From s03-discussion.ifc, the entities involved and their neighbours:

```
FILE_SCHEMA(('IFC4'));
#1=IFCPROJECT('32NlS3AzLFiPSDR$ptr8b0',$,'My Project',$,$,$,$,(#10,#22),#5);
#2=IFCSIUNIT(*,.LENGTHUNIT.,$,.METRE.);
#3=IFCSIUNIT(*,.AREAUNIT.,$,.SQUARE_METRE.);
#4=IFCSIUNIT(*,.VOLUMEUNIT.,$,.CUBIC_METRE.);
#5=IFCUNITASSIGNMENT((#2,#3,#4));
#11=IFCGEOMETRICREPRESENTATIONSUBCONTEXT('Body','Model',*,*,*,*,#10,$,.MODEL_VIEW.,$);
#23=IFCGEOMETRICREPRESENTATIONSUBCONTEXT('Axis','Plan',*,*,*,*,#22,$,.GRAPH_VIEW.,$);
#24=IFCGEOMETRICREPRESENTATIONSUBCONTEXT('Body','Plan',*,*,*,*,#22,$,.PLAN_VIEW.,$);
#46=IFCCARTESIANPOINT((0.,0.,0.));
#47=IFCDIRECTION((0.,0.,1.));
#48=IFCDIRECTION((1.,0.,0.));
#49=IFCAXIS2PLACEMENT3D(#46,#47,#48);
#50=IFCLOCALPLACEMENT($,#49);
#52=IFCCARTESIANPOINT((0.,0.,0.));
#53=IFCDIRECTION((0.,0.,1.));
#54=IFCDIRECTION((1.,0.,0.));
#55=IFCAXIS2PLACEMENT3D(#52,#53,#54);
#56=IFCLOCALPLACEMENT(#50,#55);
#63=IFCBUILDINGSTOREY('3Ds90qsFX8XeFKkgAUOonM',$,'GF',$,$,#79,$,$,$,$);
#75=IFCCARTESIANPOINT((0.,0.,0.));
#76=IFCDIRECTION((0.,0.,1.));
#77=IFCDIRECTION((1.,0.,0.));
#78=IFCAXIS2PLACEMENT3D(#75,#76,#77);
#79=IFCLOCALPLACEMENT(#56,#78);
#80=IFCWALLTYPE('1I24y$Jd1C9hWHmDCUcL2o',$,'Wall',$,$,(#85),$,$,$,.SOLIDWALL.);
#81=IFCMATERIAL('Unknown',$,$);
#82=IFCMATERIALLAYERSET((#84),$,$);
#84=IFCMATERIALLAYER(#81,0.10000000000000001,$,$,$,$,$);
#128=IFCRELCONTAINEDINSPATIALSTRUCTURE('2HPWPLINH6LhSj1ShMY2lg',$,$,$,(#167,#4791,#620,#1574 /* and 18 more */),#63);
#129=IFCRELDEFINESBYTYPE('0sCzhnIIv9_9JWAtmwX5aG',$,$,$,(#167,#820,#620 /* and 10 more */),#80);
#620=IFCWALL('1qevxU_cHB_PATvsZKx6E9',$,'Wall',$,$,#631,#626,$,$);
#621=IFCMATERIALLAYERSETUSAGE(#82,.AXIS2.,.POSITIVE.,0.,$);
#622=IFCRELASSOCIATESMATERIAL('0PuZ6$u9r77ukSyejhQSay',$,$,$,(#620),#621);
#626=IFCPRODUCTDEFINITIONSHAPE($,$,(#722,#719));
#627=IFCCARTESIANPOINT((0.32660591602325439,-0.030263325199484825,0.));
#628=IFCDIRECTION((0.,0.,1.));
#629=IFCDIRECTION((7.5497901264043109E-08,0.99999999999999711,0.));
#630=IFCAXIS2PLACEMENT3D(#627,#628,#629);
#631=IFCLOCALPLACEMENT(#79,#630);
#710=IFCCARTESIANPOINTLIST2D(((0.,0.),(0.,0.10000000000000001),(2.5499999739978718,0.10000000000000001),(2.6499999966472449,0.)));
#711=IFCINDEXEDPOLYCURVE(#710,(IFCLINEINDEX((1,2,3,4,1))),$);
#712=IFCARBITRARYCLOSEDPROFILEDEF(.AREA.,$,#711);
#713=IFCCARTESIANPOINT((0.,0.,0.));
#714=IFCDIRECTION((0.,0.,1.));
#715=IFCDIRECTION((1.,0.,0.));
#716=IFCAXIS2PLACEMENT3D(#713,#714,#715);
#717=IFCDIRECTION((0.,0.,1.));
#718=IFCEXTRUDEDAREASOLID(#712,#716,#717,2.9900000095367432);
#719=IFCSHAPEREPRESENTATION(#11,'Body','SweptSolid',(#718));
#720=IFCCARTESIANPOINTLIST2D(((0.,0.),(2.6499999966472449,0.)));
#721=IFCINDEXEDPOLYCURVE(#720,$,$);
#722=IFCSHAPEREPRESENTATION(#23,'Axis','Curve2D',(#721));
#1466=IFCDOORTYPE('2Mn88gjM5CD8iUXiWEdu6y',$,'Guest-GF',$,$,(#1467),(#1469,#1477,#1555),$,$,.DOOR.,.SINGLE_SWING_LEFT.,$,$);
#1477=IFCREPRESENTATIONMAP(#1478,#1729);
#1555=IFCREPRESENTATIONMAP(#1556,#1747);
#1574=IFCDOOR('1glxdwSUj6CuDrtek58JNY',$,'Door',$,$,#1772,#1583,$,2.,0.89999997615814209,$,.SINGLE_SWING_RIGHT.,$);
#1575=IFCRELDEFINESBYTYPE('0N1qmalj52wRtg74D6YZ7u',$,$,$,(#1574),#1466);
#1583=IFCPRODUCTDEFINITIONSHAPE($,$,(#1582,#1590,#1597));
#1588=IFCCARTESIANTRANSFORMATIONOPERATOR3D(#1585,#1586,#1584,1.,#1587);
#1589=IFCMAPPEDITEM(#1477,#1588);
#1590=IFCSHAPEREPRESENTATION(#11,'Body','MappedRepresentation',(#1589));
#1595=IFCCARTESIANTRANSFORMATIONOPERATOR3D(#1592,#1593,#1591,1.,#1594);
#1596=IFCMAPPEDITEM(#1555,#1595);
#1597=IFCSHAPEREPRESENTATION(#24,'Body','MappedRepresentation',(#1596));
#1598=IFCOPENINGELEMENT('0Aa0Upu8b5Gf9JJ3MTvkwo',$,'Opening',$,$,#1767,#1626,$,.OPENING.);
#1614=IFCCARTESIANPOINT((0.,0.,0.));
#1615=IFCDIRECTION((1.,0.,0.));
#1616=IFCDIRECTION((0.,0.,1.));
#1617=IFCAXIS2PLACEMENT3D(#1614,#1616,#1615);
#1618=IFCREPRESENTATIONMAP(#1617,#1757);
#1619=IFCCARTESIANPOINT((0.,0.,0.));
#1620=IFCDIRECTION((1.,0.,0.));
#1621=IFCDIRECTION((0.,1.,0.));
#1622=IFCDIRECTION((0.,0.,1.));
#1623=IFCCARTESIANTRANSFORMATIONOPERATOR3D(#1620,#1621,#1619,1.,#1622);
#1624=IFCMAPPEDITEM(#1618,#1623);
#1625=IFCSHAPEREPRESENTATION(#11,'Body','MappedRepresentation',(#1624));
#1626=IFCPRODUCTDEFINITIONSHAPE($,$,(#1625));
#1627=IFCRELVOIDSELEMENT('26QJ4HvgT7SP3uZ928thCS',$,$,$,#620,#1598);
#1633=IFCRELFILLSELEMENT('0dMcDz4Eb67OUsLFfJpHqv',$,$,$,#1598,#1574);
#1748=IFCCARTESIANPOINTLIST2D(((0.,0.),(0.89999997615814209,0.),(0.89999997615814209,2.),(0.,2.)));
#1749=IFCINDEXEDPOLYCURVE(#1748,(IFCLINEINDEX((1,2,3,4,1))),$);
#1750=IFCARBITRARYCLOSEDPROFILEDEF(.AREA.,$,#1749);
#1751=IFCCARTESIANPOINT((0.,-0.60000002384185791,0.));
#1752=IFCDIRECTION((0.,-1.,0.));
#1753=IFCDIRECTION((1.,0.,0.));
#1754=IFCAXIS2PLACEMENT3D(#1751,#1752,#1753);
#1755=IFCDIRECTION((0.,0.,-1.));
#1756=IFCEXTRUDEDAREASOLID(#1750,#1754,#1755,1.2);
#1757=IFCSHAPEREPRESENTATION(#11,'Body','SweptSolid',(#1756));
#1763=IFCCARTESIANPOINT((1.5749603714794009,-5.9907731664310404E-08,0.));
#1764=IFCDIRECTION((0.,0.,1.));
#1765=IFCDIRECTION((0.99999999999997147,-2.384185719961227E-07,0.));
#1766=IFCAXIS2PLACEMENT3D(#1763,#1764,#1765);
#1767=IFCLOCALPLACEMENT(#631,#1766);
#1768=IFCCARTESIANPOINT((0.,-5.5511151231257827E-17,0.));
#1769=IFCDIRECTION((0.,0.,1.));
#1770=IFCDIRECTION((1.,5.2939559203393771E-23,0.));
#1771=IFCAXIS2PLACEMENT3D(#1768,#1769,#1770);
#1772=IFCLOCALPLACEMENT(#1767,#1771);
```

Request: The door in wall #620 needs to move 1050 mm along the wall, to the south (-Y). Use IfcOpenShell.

```python
import ifcopenshell
import ifcopenshell.api.geometry
import ifcopenshell.util.placement

model = ifcopenshell.open("s03-discussion.ifc")

door = model.by_guid("1glxdwSUj6CuDrtek58JNY")
opening = door.FillsVoids[0].RelatingOpeningElement
wall = opening.VoidsElements[0].RelatingBuildingElement

wall_matrix = ifcopenshell.util.placement.get_local_placement(wall.ObjectPlacement)
shift = wall_matrix[:3, 0] * -1.05
before = ifcopenshell.util.placement.get_local_placement(door.ObjectPlacement)[:3, 3].copy()

# The door is placed relative to its opening, so it follows when the opening moves.
matrix = ifcopenshell.util.placement.get_local_placement(opening.ObjectPlacement)
matrix[:3, 3] += shift
ifcopenshell.api.geometry.edit_object_placement(
    model, product=opening, matrix=matrix, is_si=False, should_transform_children=True
)

after = ifcopenshell.util.placement.get_local_placement(door.ObjectPlacement)[:3, 3]
print("door moved by", (after - before).round(3) + 0.0)

model.write("s03-discussion_updated.ifc")
```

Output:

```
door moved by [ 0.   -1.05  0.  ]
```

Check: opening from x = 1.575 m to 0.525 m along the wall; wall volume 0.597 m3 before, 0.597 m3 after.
